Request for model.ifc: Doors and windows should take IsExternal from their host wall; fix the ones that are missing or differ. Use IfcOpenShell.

First a look at what the model holds.

```python
import ifcopenshell
import ifcopenshell.util.element

model = ifcopenshell.open("model.ifc")
print(model.schema)
seen = {}
for e in model.by_type("IfcDoor") + model.by_type("IfcWindow"):
    if not e.FillsVoids:
        continue
    host = e.FillsVoids[0].RelatingOpeningElement.VoidsElements[0].RelatingBuildingElement
    own = ifcopenshell.util.element.get_pset(e, f"Pset_{e.is_a()[3:].removesuffix('StandardCase')}Common", "IsExternal")
    wall = ifcopenshell.util.element.get_pset(host, "Pset_WallCommon", "IsExternal")
    seen[e.is_a(), own, wall] = seen.get((e.is_a(), own, wall), 0) + 1
for (cls, own, wall), count in sorted(seen.items(), key=str):
    print(count, cls, "IsExternal:", own, "| host wall:", wall)
```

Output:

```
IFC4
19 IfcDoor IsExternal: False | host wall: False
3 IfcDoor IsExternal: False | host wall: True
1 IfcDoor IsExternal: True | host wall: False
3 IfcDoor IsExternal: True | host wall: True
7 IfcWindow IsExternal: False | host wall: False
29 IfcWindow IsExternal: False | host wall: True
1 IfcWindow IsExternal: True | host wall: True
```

```python
import ifcopenshell
import ifcopenshell.api.pset
import ifcopenshell.util.element

model = ifcopenshell.open("model.ifc")

count = 0
for ifc_class, pset_name in (("IfcDoor", "Pset_DoorCommon"), ("IfcWindow", "Pset_WindowCommon")):
    for e in model.by_type(ifc_class):
        if not e.FillsVoids:
            continue
        host = e.FillsVoids[0].RelatingOpeningElement.VoidsElements[0].RelatingBuildingElement
        external = ifcopenshell.util.element.get_pset(host, "Pset_WallCommon", "IsExternal")
        if external is None or ifcopenshell.util.element.get_pset(e, pset_name, "IsExternal") == external:
            continue
        pset = ifcopenshell.api.pset.add_pset(model, product=e, name=pset_name)
        ifcopenshell.api.pset.edit_pset(model, pset=pset, properties={"IsExternal": external})
        count += 1

print(count, "updated")

model.write("model_rev.ifc")
```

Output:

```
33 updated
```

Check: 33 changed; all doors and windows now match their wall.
